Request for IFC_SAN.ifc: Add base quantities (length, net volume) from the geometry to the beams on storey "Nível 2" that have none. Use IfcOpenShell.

First a look at what the model holds.

```python
import ifcopenshell
import ifcopenshell.util.element
import ifcopenshell.util.unit

model = ifcopenshell.open("IFC_SAN.ifc")
print(model.schema)
for unit_type in ("LENGTHUNIT", "AREAUNIT", "VOLUMEUNIT"):
    print(unit_type, ifcopenshell.util.unit.calculate_unit_scale(model, unit_type))
storey = next(s for s in model.by_type("IfcBuildingStorey") if s.Name == "Nível 2")
beams = [e for e in ifcopenshell.util.element.get_decomposition(storey) if e.is_a("IfcBeam")]
for e in sorted(beams, key=lambda e: e.id()):
    print(e.id(), e.is_a(), e.Name, list(ifcopenshell.util.element.get_psets(e, qtos_only=True)), sep=" | ")
```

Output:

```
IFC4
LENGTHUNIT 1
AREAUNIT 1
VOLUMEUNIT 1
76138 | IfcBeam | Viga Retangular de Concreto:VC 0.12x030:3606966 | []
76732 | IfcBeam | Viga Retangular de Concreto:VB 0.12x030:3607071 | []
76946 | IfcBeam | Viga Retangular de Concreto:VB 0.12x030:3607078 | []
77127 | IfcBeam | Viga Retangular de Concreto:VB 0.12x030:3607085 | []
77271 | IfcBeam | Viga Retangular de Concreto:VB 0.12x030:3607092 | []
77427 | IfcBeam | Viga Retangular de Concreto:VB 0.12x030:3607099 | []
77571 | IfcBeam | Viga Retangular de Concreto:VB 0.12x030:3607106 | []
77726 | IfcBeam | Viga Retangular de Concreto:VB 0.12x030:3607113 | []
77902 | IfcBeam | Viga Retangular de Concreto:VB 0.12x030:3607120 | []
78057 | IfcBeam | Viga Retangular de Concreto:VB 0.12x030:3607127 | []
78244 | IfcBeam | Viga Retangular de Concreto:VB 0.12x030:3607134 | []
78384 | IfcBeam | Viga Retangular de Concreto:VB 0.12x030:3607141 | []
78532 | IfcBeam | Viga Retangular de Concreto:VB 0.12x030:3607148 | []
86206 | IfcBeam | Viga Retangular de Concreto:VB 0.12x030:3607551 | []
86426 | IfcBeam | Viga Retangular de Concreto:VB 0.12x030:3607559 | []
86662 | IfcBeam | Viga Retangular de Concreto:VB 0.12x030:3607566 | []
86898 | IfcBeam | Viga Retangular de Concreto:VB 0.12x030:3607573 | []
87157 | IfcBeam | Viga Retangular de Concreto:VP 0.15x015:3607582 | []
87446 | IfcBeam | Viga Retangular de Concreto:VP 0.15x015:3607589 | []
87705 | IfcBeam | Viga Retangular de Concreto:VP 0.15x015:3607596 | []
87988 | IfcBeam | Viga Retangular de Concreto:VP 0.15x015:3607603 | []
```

```python
import ifcopenshell
import ifcopenshell.api.pset
import ifcopenshell.geom
import ifcopenshell.util.element
import ifcopenshell.util.shape
import ifcopenshell.util.unit

model = ifcopenshell.open("IFC_SAN.ifc")
unit_scale = ifcopenshell.util.unit.calculate_unit_scale(model)
volume_scale = ifcopenshell.util.unit.calculate_unit_scale(model, "VOLUMEUNIT")
settings = ifcopenshell.geom.settings()

storey = next(s for s in model.by_type("IfcBuildingStorey") if s.Name == "Nível 2")
beams = [e for e in ifcopenshell.util.element.get_decomposition(storey) if e.is_a("IfcBeam")]

for e in sorted(beams, key=lambda e: e.id()):
    if ifcopenshell.util.element.get_psets(e, qtos_only=True, should_inherit=False):
        continue
    # Geometry comes back in metres, in the element's own axes.
    shape = ifcopenshell.geom.create_shape(settings, e)
    values = {
        "Length": ifcopenshell.util.shape.get_max_xyz(shape.geometry) / unit_scale,
        "NetVolume": ifcopenshell.util.shape.get_volume(shape.geometry) / volume_scale,
    }
    qto = ifcopenshell.api.pset.add_qto(model, product=e, name="Qto_BeamBaseQuantities")
    ifcopenshell.api.pset.edit_qto(model, qto=qto, properties=values)
    print(e.id(), {k: round(v, 3) for k, v in values.items()})

model.write("IFC_SAN_v2.ifc")
```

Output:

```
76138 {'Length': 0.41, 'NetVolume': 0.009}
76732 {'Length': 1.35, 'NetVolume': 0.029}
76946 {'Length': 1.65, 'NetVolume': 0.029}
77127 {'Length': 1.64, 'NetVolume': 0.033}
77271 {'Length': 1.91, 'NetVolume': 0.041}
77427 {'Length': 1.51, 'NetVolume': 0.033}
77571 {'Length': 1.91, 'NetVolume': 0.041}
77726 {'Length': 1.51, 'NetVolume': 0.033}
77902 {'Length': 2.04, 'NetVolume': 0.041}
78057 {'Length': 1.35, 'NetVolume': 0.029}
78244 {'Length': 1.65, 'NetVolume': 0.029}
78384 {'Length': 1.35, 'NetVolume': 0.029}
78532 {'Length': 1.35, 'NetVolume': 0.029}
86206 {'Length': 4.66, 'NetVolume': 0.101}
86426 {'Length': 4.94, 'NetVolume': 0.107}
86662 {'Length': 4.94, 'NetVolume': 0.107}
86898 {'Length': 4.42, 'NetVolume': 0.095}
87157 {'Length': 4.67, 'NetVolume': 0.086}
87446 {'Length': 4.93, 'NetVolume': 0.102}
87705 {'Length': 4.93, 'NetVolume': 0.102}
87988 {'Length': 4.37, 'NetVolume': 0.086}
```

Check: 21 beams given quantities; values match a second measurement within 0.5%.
